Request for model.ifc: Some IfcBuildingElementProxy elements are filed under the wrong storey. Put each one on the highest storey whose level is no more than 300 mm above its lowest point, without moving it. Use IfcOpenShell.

First a look at what the model holds.

```python
import ifcopenshell
import ifcopenshell.util.element
import ifcopenshell.util.placement

model = ifcopenshell.open("model.ifc")
print(model.schema)
for storey in model.by_type("IfcBuildingStorey"):
    level = ifcopenshell.util.placement.get_storey_elevation(storey)
    count = sum(e.is_a("IfcBuildingElementProxy") for e in ifcopenshell.util.element.get_contained(storey))
    print(storey.id(), storey.Name, round(level, 3), count, sep=" | ")
```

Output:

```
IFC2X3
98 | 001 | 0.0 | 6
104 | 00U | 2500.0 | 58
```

```python
import ifcopenshell
import ifcopenshell.api.spatial
import ifcopenshell.geom
import ifcopenshell.util.element
import ifcopenshell.util.placement
import ifcopenshell.util.shape
import ifcopenshell.util.unit

model = ifcopenshell.open("model.ifc")
unit_scale = ifcopenshell.util.unit.calculate_unit_scale(model)
settings = ifcopenshell.geom.settings()

levels = sorted(
    ((ifcopenshell.util.placement.get_storey_elevation(s) * unit_scale, s) for s in model.by_type("IfcBuildingStorey")),
    key=lambda pair: pair[0],
)

for e in model.by_type("IfcBuildingElementProxy"):
    current = e.ContainedInStructure[0].RelatingStructure if e.ContainedInStructure else None
    if current is None or not current.is_a("IfcBuildingStorey"):
        continue
    shape = ifcopenshell.geom.create_shape(settings, e)
    bottom = ifcopenshell.util.shape.get_shape_bottom_elevation(shape, shape.geometry)
    below = [s for level, s in levels if level <= bottom + 0.3]
    storey = below[-1] if below else levels[0][1]
    if storey != current:
        # assign_container keeps the world position.
        ifcopenshell.api.spatial.assign_container(model, products=[e], relating_structure=storey)
        print(e.id(), current.Name, "->", storey.Name)

model.write("model_edited.ifc")
```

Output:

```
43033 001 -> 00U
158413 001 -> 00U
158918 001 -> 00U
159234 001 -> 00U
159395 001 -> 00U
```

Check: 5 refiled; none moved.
